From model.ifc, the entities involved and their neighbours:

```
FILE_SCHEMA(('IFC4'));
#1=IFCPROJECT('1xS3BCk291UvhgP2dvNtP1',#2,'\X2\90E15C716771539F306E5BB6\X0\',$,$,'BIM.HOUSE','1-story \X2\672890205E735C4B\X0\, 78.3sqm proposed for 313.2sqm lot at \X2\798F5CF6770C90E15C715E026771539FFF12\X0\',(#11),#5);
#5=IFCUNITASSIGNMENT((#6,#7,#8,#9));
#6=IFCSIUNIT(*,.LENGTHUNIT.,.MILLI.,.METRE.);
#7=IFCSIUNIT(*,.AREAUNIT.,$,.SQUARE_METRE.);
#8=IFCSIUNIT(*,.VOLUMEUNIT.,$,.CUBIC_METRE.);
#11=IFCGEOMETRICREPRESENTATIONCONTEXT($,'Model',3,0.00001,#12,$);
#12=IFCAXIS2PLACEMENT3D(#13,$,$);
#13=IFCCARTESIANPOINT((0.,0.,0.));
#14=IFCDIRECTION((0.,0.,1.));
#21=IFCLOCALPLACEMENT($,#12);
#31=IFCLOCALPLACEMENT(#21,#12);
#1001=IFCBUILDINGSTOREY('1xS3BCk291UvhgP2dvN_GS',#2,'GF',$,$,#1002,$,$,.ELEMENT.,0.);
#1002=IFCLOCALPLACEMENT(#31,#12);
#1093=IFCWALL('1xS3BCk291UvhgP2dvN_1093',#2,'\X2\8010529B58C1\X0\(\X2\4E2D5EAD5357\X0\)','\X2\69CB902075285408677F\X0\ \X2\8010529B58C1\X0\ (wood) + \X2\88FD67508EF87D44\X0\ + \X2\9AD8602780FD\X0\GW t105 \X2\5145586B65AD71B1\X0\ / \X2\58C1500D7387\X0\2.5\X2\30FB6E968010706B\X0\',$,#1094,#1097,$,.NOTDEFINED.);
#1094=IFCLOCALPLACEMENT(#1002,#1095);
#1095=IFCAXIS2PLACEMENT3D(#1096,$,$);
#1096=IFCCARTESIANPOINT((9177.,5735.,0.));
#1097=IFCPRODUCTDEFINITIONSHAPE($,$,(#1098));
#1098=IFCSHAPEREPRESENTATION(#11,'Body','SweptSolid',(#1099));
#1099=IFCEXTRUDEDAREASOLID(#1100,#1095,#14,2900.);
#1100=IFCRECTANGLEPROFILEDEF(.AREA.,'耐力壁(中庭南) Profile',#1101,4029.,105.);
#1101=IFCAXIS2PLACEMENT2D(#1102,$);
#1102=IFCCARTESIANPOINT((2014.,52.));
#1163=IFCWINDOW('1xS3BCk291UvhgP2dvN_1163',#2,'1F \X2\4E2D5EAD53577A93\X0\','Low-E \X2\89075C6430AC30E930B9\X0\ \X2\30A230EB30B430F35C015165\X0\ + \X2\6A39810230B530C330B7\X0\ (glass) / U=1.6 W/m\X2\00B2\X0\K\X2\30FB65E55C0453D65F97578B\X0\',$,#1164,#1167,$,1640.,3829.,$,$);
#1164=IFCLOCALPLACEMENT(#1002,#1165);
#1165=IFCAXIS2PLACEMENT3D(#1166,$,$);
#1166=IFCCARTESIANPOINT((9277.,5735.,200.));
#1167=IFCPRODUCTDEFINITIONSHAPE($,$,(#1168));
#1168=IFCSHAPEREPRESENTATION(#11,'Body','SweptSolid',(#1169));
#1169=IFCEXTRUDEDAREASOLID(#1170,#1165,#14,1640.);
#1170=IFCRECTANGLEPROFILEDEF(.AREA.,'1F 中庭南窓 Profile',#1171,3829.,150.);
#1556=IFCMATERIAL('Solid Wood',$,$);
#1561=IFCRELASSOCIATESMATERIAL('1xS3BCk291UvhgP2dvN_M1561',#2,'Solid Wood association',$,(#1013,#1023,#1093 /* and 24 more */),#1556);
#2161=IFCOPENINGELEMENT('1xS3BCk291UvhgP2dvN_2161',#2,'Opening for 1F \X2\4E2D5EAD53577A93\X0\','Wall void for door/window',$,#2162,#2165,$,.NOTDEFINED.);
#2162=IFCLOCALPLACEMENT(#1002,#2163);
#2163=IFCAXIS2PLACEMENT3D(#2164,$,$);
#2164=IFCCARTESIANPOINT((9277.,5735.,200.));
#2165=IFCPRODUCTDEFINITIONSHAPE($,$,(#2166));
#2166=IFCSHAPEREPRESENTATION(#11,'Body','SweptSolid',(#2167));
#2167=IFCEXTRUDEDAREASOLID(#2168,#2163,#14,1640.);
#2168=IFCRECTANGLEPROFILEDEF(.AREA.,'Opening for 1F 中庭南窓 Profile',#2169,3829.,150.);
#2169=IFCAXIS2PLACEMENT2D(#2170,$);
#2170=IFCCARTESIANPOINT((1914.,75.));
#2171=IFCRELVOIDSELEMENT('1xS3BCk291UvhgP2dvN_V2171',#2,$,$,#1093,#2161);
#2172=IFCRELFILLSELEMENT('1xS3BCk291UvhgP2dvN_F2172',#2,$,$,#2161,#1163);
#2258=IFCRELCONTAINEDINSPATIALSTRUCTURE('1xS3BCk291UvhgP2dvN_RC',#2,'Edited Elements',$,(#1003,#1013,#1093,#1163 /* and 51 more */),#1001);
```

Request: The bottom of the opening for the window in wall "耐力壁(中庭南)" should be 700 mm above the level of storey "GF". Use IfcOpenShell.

```python
import numpy as np
import ifcopenshell
import ifcopenshell.api.geometry
import ifcopenshell.geom
import ifcopenshell.util.element
import ifcopenshell.util.placement
import ifcopenshell.util.shape
import ifcopenshell.util.unit

model = ifcopenshell.open("model.ifc")
unit_scale = ifcopenshell.util.unit.calculate_unit_scale(model)

window = model.by_guid("1xS3BCk291UvhgP2dvN_1163")
opening = window.FillsVoids[0].RelatingOpeningElement
storey = ifcopenshell.util.element.get_container(window, ifc_class="IfcBuildingStorey")
level = ifcopenshell.util.placement.get_local_placement(storey.ObjectPlacement)[2, 3]

# The opening's origin need not be at the sill, so measure its lowest point.
shape = ifcopenshell.geom.create_shape(ifcopenshell.geom.settings(), opening)
bottom = ifcopenshell.util.shape.get_shape_bottom_elevation(shape, shape.geometry) / unit_scale
dz = level + 0.7 / unit_scale - bottom

shift = np.array([0.0, 0.0, dz])
# The window is not placed relative to its opening, so move both.
for product in (opening, window):
    matrix = ifcopenshell.util.placement.get_local_placement(product.ObjectPlacement)
    matrix[:3, 3] += shift
    ifcopenshell.api.geometry.edit_object_placement(model, product=product, matrix=matrix, is_si=False)

print(f"moved by {dz * unit_scale:+.3f} m")

model.write("model_v2.ifc")
```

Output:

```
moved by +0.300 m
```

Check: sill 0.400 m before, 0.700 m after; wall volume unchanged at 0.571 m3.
